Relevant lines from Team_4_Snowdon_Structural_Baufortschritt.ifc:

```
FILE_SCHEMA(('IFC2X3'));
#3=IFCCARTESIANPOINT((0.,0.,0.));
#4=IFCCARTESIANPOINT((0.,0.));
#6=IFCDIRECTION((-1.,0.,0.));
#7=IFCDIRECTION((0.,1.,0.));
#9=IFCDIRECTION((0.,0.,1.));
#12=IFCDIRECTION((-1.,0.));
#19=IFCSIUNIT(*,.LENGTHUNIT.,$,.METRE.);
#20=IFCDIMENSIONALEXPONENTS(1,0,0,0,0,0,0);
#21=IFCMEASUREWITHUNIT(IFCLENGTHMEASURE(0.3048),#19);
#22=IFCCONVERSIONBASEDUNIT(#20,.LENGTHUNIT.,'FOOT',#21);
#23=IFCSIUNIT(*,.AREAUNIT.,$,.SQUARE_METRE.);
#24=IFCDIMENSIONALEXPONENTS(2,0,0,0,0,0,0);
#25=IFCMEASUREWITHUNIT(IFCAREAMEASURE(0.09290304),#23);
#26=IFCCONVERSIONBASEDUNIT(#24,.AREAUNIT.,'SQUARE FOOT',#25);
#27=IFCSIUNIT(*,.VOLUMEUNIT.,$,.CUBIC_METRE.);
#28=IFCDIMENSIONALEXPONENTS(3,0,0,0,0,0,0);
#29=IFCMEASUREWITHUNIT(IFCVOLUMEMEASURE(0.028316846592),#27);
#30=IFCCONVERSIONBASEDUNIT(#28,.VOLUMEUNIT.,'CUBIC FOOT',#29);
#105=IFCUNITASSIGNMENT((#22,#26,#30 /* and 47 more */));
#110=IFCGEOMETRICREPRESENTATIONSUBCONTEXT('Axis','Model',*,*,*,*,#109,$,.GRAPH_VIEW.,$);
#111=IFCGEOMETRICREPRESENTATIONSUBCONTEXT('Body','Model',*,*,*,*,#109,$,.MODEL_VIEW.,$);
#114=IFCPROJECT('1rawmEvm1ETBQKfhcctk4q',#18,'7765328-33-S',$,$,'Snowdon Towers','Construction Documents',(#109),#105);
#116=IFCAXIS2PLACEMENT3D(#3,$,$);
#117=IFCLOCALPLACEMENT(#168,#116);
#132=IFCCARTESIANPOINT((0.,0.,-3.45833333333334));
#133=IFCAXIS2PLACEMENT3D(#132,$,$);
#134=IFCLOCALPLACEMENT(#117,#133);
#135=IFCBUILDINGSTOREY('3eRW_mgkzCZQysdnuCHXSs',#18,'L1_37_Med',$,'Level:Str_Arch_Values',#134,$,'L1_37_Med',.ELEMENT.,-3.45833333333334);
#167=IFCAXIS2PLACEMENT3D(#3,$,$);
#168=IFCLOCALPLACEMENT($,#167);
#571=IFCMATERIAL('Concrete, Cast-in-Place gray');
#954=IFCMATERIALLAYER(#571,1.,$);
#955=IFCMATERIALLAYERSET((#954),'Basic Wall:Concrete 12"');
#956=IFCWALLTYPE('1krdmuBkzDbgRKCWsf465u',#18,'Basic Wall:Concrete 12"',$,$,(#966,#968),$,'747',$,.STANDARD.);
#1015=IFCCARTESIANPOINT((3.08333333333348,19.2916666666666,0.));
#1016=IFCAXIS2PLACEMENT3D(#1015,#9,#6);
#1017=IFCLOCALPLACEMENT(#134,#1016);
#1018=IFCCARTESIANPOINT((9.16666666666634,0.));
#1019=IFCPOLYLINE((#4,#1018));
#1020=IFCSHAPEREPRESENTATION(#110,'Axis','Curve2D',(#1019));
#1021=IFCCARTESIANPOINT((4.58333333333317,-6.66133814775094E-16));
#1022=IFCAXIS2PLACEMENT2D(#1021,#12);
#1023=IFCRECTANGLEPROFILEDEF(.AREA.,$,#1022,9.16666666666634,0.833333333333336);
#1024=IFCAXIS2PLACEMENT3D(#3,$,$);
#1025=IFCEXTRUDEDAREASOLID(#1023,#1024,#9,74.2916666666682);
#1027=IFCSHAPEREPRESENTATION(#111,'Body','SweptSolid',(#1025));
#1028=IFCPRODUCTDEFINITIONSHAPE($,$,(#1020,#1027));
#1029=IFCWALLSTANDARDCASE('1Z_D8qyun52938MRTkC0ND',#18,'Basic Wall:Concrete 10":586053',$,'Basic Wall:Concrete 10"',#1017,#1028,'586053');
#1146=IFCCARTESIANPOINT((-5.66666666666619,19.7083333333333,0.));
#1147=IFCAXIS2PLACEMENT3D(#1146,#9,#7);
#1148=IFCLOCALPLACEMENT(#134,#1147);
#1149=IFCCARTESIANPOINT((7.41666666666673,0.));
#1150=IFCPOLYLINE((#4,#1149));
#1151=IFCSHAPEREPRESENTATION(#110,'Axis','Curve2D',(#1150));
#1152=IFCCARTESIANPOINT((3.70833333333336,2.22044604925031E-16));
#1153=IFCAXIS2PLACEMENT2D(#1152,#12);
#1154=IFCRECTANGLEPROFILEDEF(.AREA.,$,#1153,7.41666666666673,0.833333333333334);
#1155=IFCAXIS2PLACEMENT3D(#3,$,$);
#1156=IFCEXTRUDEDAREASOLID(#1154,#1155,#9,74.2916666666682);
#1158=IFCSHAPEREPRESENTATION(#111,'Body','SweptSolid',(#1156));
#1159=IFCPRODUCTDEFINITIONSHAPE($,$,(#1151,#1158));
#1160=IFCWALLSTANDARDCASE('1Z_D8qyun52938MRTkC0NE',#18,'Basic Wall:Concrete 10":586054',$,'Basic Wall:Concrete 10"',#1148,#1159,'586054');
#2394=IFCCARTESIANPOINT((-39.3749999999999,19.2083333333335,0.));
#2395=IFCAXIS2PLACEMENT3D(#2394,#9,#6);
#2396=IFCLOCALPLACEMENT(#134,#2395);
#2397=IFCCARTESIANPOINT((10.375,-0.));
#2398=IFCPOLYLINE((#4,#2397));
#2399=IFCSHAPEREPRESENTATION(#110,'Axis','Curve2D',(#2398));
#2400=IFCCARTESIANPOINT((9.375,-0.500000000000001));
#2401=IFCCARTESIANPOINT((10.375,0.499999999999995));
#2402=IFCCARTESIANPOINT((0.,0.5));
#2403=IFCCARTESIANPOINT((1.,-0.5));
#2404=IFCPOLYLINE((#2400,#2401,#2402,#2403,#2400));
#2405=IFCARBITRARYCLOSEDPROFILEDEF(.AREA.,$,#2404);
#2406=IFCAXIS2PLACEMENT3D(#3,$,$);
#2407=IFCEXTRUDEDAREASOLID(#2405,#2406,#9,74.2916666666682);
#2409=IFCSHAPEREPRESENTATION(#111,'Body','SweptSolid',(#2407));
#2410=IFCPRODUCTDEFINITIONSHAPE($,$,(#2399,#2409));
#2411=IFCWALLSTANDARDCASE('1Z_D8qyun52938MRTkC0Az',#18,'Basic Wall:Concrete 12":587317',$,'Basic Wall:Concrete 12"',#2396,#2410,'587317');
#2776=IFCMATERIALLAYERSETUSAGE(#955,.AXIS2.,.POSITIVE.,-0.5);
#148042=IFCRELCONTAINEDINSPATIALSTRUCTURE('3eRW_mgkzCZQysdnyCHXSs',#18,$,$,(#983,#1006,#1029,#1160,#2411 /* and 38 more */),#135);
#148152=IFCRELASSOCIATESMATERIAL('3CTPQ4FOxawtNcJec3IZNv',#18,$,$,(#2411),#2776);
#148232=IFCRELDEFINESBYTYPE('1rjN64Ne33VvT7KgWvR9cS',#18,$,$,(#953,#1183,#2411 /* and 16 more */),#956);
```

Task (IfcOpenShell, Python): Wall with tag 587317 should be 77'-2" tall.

```python
import ifcopenshell
import ifcopenshell.geom
import ifcopenshell.util.representation
import ifcopenshell.util.shape
import ifcopenshell.util.unit

model = ifcopenshell.open("Team_4_Snowdon_Structural_Baufortschritt.ifc")
unit_scale = ifcopenshell.util.unit.calculate_unit_scale(model)
settings = ifcopenshell.geom.settings()


def volume(element):
    """Net volume in cubic metres, openings subtracted."""
    shape = ifcopenshell.geom.create_shape(settings, element)
    return ifcopenshell.util.shape.get_volume(shape.geometry)


wall = model.by_guid("1Z_D8qyun52938MRTkC0Az")
before = volume(wall)

body = ifcopenshell.util.representation.get_representation(wall, "Model", "Body")
solid = body.Items[0]
old_height = solid.Depth
solid.Depth = 926 * 0.0254 / unit_scale
after = volume(wall)

print(f"height {old_height:g} -> {solid.Depth:g}, volume {before:.3f} -> {after:.3f} m3")

model.write("Team_4_Snowdon_Structural_Baufortschritt_v2.ifc")
```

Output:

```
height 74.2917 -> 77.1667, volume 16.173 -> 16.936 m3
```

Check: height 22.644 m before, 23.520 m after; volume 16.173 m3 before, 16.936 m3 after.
